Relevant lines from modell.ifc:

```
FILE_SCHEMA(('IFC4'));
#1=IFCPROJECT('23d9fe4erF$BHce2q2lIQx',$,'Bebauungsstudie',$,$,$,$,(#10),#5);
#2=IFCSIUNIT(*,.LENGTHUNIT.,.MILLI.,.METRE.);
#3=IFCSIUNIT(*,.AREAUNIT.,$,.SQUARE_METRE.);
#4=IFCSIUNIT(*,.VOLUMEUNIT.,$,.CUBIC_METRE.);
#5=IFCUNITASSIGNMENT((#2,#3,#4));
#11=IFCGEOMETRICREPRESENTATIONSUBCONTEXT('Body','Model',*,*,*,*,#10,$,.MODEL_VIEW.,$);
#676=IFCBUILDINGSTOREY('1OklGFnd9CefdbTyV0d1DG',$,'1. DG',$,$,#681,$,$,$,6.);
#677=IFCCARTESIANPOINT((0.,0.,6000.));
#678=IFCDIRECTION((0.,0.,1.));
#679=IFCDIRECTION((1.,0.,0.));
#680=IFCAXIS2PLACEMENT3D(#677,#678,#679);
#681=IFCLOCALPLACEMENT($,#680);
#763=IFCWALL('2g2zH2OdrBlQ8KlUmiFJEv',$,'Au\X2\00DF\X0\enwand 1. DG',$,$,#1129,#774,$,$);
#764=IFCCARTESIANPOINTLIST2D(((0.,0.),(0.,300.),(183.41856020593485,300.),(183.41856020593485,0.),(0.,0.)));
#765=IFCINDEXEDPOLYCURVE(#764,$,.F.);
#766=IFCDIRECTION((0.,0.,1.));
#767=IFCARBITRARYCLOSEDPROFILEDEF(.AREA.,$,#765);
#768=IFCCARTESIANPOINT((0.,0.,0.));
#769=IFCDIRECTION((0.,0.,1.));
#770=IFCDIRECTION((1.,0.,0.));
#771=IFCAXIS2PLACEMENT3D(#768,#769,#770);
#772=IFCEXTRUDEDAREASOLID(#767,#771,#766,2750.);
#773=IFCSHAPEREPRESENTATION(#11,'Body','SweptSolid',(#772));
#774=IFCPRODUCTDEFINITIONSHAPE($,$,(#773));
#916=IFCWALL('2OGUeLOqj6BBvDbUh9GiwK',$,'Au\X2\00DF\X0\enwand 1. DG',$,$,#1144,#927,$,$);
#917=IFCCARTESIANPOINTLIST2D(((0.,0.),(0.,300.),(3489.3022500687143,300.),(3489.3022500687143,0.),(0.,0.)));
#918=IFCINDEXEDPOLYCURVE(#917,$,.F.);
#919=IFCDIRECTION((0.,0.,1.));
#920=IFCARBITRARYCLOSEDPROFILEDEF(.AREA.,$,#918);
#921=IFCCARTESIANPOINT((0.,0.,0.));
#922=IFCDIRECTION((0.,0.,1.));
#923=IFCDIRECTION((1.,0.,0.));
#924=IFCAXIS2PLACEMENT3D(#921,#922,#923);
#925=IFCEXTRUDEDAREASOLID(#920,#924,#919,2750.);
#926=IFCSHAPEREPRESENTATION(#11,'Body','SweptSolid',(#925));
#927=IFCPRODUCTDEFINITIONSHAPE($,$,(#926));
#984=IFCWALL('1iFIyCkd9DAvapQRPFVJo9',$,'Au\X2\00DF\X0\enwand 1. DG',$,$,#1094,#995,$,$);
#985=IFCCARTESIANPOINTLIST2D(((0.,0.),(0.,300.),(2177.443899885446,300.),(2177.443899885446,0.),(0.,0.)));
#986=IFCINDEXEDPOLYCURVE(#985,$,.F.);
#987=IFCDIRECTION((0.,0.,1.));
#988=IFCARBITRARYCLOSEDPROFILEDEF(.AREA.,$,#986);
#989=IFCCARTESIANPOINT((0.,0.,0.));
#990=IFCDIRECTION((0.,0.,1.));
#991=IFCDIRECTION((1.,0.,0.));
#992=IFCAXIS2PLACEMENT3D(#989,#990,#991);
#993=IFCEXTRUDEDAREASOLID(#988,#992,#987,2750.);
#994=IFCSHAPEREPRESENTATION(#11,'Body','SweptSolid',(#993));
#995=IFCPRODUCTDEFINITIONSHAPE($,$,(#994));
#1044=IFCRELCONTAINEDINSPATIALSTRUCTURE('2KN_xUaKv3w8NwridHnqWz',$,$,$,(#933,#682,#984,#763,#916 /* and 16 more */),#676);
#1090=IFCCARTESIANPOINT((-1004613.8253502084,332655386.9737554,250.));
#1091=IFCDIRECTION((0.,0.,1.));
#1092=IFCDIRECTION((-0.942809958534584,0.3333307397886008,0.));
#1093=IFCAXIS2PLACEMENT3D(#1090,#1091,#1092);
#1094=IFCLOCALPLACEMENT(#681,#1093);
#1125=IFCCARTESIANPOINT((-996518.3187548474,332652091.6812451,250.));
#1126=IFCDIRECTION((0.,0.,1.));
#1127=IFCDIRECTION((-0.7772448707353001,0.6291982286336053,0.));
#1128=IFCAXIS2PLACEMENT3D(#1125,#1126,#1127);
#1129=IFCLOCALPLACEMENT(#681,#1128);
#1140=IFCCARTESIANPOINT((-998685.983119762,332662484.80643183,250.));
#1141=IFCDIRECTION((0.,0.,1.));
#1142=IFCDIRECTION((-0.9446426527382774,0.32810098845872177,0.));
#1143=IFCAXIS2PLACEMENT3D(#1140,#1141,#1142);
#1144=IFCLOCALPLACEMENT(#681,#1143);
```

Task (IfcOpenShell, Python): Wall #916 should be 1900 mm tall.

```python
import ifcopenshell
import ifcopenshell.geom
import ifcopenshell.util.representation
import ifcopenshell.util.shape
import ifcopenshell.util.unit

model = ifcopenshell.open("modell.ifc")
unit_scale = ifcopenshell.util.unit.calculate_unit_scale(model)
settings = ifcopenshell.geom.settings()


def volume(element):
    """Net volume in cubic metres, openings subtracted."""
    shape = ifcopenshell.geom.create_shape(settings, element)
    return ifcopenshell.util.shape.get_volume(shape.geometry)


wall = model.by_id(916)
before = volume(wall)

body = ifcopenshell.util.representation.get_representation(wall, "Model", "Body")
solid = body.Items[0]
old_height = solid.Depth
solid.Depth = 1.9 / unit_scale
after = volume(wall)

print(f"height {old_height:g} -> {solid.Depth:g}, volume {before:.3f} -> {after:.3f} m3")

model.write("modell_v2.ifc")
```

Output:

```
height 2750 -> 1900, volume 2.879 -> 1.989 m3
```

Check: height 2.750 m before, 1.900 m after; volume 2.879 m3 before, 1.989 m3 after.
